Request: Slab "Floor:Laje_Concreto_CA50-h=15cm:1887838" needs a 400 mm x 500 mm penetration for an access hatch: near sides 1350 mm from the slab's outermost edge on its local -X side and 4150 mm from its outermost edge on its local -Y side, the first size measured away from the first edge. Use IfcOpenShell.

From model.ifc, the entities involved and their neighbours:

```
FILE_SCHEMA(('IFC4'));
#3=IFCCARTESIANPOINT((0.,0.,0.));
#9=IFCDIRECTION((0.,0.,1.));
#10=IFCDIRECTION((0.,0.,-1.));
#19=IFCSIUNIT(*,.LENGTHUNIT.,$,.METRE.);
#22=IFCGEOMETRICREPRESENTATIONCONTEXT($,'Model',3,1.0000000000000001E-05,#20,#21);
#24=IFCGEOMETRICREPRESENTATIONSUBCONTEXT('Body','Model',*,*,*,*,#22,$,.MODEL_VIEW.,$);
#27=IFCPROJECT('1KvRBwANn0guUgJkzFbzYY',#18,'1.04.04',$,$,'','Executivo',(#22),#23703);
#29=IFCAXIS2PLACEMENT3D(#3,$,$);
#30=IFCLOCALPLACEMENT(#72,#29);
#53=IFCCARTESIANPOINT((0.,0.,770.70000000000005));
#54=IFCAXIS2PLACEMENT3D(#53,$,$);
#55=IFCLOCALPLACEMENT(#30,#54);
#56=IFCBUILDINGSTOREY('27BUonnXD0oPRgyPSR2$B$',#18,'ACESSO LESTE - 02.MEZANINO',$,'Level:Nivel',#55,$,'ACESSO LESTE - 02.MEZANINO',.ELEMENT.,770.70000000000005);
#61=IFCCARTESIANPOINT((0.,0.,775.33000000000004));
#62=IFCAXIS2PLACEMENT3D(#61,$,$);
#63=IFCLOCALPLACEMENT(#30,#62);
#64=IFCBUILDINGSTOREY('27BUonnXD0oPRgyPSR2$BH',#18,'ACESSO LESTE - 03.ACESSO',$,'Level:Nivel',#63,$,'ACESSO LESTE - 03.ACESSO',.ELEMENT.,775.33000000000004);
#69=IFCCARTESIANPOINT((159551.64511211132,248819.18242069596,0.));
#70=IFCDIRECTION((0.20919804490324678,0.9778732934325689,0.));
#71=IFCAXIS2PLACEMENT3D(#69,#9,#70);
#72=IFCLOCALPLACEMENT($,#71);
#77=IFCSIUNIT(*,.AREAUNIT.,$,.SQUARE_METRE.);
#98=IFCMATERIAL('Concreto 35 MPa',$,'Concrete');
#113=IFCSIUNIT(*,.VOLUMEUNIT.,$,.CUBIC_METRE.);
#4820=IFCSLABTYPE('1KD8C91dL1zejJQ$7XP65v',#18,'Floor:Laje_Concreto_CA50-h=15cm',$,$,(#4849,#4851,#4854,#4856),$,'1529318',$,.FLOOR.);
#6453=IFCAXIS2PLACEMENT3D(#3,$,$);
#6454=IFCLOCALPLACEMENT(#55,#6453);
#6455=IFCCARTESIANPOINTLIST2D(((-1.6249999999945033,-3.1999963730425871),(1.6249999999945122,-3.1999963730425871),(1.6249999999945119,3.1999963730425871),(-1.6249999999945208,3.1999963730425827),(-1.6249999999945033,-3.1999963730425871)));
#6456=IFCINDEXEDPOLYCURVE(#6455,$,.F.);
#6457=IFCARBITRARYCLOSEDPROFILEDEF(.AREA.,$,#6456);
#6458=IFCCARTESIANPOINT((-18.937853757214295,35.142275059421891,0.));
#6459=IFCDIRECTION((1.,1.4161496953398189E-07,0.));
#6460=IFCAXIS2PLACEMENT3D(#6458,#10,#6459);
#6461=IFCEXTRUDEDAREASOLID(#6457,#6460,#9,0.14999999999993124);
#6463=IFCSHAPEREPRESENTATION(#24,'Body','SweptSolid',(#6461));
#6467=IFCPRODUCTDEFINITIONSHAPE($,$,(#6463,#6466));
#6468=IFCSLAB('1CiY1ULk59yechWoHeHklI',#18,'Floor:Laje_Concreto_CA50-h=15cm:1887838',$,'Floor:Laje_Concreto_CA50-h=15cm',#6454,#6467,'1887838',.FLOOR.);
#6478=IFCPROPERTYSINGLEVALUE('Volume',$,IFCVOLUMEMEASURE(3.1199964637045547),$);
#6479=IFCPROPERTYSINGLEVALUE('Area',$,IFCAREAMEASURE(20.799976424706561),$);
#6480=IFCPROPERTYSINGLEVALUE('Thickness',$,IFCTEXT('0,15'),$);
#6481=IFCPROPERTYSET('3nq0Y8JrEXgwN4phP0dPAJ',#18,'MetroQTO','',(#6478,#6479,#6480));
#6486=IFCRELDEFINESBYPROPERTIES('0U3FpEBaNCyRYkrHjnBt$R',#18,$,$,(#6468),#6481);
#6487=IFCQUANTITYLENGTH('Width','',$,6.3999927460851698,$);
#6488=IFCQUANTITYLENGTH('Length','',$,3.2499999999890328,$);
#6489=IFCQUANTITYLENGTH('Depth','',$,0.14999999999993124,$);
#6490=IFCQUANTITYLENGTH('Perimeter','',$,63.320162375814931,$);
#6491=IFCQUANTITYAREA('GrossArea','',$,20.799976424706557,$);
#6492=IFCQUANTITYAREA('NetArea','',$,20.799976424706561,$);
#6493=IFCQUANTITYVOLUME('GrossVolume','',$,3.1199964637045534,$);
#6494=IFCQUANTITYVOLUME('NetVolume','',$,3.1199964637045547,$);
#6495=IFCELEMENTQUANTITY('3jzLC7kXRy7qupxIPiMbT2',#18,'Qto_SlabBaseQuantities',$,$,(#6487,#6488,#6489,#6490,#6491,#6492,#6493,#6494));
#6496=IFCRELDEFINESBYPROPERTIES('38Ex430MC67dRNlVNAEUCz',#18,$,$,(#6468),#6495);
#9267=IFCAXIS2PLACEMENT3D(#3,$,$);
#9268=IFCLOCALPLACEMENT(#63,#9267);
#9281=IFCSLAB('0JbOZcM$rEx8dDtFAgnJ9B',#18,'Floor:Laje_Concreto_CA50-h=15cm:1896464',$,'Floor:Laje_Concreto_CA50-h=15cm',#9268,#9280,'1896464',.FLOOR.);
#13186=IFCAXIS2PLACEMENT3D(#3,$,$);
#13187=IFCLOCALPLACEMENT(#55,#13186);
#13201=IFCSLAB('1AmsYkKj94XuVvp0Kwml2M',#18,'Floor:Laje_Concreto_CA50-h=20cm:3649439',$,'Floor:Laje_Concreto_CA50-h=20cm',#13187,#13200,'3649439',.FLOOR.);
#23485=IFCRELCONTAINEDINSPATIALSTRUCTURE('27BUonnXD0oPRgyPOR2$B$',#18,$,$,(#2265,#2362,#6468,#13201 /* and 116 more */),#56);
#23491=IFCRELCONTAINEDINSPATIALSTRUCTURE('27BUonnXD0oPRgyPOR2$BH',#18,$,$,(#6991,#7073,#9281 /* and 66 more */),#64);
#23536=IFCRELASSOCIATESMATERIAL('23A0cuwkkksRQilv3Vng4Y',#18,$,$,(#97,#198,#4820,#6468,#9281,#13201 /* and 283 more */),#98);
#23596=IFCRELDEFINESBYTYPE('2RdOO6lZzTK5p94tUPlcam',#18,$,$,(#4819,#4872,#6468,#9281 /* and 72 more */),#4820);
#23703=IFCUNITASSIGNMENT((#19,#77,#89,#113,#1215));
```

```python
import numpy as np
import ifcopenshell
import ifcopenshell.api.feature
import ifcopenshell.api.geometry
import ifcopenshell.api.pset
import ifcopenshell.api.root
import ifcopenshell.geom
import ifcopenshell.util.element
import ifcopenshell.util.placement
import ifcopenshell.util.representation
import ifcopenshell.util.shape
import ifcopenshell.util.unit

model = ifcopenshell.open("model.ifc")
unit_scale = ifcopenshell.util.unit.calculate_unit_scale(model)
area_scale = ifcopenshell.util.unit.calculate_unit_scale(model, "AREAUNIT")
volume_scale = ifcopenshell.util.unit.calculate_unit_scale(model, "VOLUMEUNIT")
settings = ifcopenshell.geom.settings()


def volume(element):
    """Net volume in cubic metres, openings subtracted."""
    shape = ifcopenshell.geom.create_shape(settings, element)
    return ifcopenshell.util.shape.get_volume(shape.geometry)


slab = model.by_guid("1CiY1ULk59yechWoHeHklI")
before = volume(slab)

# Extent in the slab's own axes, in metres. The edges named are its -X and -Y sides.
slab_shape = ifcopenshell.geom.create_shape(settings, slab)
vertices = ifcopenshell.util.shape.get_vertices(slab_shape.geometry)
x_min, y_min, bottom = vertices.min(axis=0)
top = vertices[:, 2].max()

opening = ifcopenshell.api.root.create_entity(model, ifc_class="IfcOpeningElement", name="Access hatch opening", predefined_type="OPENING")
context = ifcopenshell.util.representation.get_context(model, "Model", "Body", "MODEL_VIEW")
width, depth = 0.4, 0.5
outline = [(0.0, 0.0), (width, 0.0), (width, depth), (0.0, depth), (0.0, 0.0)]
# Overshoot both faces by 50 mm so the cut is clean.
shape = ifcopenshell.api.geometry.add_slab_representation(
    model, context=context, depth=top - bottom + 0.1, polyline=outline
)
ifcopenshell.api.geometry.assign_representation(model, product=opening, representation=shape)

matrix = ifcopenshell.util.placement.get_local_placement(slab.ObjectPlacement)
matrix[:, 3] = matrix @ np.append(np.array([x_min + 1.35, y_min + 4.15, bottom - 0.05]) / unit_scale, 1.0)
ifcopenshell.api.geometry.edit_object_placement(model, product=opening, matrix=matrix, is_si=False)
ifcopenshell.api.feature.add_feature(model, feature=opening, element=slab)

after = volume(slab)

# Update the slab's stored quantities.
pset = model.by_id(ifcopenshell.util.element.get_pset(slab, "MetroQTO", should_inherit=False)["id"])
ifcopenshell.api.pset.edit_pset(model, pset=pset, properties={
    "Volume": model.create_entity("IfcVolumeMeasure", after / volume_scale),
    "Area": model.create_entity("IfcAreaMeasure", after / (top - bottom) / area_scale),
})
qto = model.by_id(ifcopenshell.util.element.get_pset(slab, "Qto_SlabBaseQuantities", should_inherit=False)["id"])
ifcopenshell.api.pset.edit_qto(model, qto=qto, properties={
    "NetArea": after / (top - bottom) / area_scale,
    "NetVolume": after / volume_scale,
})

print(f"slab volume {before:.3f} -> {after:.3f} m3")

model.write("model-out.ifc")
```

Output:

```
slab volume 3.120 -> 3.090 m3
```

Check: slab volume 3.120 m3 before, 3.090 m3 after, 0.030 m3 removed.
